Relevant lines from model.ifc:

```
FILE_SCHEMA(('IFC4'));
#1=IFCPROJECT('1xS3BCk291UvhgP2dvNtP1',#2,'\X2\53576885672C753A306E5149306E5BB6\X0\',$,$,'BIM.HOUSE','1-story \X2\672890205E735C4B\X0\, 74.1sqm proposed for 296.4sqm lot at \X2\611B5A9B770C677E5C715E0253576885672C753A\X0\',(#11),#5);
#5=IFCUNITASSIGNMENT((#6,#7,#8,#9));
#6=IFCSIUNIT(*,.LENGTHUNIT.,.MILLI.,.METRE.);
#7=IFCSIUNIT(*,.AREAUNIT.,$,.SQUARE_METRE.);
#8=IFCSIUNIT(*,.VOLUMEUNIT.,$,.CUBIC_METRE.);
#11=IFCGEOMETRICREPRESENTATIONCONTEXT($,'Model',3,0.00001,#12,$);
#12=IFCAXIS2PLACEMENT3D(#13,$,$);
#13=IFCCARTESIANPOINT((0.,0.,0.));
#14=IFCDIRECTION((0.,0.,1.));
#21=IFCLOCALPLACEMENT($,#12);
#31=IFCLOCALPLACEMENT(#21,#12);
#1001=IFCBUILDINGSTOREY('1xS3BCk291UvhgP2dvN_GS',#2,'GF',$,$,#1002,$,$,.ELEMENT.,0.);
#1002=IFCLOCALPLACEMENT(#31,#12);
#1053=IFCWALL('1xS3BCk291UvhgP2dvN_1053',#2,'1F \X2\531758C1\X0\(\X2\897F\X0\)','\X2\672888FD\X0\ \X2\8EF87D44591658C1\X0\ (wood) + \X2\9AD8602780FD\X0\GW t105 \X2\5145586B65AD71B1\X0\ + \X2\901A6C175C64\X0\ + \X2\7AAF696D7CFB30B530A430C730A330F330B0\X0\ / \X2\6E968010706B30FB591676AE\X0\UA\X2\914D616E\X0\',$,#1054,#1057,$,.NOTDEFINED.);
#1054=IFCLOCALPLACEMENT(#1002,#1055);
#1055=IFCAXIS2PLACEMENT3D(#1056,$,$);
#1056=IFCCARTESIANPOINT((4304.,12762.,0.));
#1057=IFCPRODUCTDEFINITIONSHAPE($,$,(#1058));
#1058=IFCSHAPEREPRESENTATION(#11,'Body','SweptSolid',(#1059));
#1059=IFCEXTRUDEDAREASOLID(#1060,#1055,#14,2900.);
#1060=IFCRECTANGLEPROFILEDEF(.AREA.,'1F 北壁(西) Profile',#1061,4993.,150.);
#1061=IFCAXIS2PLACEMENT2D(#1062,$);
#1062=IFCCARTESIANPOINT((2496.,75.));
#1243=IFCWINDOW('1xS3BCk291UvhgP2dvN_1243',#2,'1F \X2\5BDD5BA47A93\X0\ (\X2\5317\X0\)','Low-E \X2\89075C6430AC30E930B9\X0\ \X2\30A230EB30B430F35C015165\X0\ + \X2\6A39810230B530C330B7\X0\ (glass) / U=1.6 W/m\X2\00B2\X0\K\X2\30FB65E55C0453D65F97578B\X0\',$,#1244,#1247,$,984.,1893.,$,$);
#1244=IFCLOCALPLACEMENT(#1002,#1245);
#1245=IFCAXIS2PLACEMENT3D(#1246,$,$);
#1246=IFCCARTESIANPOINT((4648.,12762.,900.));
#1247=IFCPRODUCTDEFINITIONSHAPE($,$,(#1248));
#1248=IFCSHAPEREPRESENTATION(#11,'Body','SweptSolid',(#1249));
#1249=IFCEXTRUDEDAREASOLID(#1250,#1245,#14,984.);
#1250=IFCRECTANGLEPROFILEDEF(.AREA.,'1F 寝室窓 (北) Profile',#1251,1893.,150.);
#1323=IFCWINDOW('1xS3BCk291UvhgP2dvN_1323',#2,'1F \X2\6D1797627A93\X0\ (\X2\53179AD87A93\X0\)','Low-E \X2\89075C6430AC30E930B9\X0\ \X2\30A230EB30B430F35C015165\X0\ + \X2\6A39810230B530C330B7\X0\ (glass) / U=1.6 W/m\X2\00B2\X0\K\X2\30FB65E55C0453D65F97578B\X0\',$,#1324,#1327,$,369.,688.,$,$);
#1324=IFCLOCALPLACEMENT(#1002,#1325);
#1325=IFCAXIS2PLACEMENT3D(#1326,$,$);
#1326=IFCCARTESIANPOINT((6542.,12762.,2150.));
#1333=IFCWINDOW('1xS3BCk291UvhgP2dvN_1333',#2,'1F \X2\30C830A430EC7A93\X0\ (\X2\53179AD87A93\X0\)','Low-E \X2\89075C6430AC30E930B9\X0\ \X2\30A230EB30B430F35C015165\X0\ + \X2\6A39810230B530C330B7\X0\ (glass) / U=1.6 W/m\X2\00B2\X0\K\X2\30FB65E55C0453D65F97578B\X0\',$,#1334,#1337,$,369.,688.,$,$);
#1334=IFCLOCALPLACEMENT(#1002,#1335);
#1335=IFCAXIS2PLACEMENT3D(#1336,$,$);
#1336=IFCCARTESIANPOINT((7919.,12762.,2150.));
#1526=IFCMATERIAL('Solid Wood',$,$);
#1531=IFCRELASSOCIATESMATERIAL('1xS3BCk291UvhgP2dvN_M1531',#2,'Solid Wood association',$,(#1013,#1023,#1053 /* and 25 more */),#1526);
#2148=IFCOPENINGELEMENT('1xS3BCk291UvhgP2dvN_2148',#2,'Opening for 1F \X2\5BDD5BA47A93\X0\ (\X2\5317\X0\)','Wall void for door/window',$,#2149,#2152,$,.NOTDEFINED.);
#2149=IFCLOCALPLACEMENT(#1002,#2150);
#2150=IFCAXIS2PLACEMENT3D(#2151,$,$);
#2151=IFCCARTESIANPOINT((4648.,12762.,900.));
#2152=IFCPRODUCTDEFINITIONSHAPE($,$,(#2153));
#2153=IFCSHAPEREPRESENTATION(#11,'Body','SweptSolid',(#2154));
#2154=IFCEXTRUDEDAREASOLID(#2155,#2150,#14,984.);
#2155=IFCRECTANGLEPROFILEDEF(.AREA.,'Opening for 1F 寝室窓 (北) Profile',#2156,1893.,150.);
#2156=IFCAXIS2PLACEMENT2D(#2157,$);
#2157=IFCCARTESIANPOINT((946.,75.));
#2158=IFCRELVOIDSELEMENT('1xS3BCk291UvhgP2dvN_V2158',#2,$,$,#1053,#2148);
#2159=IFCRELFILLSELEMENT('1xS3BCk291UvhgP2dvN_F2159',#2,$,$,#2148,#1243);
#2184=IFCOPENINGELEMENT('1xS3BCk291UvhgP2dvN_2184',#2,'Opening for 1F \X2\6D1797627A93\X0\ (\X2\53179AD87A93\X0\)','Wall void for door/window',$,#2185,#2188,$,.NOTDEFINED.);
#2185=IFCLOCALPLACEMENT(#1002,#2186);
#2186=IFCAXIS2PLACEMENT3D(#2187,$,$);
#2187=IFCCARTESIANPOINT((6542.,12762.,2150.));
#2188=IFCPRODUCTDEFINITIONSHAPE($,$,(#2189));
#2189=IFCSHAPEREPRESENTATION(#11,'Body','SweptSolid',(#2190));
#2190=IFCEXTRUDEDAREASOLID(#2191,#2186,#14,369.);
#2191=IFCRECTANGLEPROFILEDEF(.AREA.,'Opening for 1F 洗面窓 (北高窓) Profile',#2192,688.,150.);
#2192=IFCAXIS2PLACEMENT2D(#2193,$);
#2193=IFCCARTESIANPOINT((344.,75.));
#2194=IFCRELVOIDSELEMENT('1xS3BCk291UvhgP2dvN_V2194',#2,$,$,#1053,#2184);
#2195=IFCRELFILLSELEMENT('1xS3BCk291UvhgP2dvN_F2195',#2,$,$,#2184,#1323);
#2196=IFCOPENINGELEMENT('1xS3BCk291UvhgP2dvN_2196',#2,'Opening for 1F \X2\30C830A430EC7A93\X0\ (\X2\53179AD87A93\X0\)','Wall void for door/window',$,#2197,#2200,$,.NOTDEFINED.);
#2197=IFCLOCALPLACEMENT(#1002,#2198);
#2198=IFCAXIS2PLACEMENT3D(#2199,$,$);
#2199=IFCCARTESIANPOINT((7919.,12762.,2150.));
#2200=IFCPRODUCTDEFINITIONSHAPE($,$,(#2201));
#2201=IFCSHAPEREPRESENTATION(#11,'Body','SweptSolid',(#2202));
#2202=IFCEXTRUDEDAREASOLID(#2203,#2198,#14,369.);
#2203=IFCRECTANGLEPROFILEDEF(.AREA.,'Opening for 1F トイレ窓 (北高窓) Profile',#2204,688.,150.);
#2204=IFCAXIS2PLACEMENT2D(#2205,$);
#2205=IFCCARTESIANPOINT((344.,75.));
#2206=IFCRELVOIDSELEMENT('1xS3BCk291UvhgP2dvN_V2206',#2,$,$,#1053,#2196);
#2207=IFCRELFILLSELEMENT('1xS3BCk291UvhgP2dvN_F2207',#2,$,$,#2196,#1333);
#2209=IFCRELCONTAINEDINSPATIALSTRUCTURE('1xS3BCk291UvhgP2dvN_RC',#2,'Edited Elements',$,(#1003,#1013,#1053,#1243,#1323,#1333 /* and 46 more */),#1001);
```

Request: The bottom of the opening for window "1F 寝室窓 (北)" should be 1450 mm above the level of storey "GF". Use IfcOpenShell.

```python
import numpy as np
import ifcopenshell
import ifcopenshell.api.geometry
import ifcopenshell.geom
import ifcopenshell.util.element
import ifcopenshell.util.placement
import ifcopenshell.util.shape
import ifcopenshell.util.unit

model = ifcopenshell.open("model.ifc")
unit_scale = ifcopenshell.util.unit.calculate_unit_scale(model)

window = model.by_id(1243)
opening = window.FillsVoids[0].RelatingOpeningElement
storey = ifcopenshell.util.element.get_container(window, ifc_class="IfcBuildingStorey")
level = ifcopenshell.util.placement.get_local_placement(storey.ObjectPlacement)[2, 3]

# The opening's origin need not be at the sill, so measure its lowest point.
shape = ifcopenshell.geom.create_shape(ifcopenshell.geom.settings(), opening)
bottom = ifcopenshell.util.shape.get_shape_bottom_elevation(shape, shape.geometry) / unit_scale
dz = level + 1450.0 - bottom

shift = np.array([0.0, 0.0, dz])
# The window is not placed relative to its opening, so move both.
for product in (opening, window):
    matrix = ifcopenshell.util.placement.get_local_placement(product.ObjectPlacement)
    matrix[:3, 3] += shift
    ifcopenshell.api.geometry.edit_object_placement(model, product=product, matrix=matrix, is_si=False)

print(f"moved by {dz * unit_scale:+.3f} m")

model.write("model_rev.ifc")
```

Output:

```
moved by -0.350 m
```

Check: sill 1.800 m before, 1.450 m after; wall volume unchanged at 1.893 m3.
